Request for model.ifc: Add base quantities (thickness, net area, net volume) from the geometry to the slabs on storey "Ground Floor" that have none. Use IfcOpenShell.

First a look at what the model holds.

```python
import ifcopenshell
import ifcopenshell.util.element
import ifcopenshell.util.unit

model = ifcopenshell.open("model.ifc")
print(model.schema)
for unit_type in ("LENGTHUNIT", "AREAUNIT", "VOLUMEUNIT"):
    print(unit_type, ifcopenshell.util.unit.calculate_unit_scale(model, unit_type))
storey = next(s for s in model.by_type("IfcBuildingStorey") if s.Name == "Ground Floor")
slabs = [e for e in ifcopenshell.util.element.get_decomposition(storey) if e.is_a("IfcSlab")]
for e in sorted(slabs, key=lambda e: e.id()):
    print(e.id(), e.is_a(), e.Name, list(ifcopenshell.util.element.get_psets(e, qtos_only=True)), sep=" | ")
```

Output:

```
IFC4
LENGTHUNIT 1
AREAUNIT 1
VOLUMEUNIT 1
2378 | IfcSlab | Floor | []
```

```python
import ifcopenshell
import ifcopenshell.api.pset
import ifcopenshell.geom
import ifcopenshell.util.element
import ifcopenshell.util.shape
import ifcopenshell.util.unit

model = ifcopenshell.open("model.ifc")
unit_scale = ifcopenshell.util.unit.calculate_unit_scale(model)
area_scale = ifcopenshell.util.unit.calculate_unit_scale(model, "AREAUNIT")
volume_scale = ifcopenshell.util.unit.calculate_unit_scale(model, "VOLUMEUNIT")
settings = ifcopenshell.geom.settings()

storey = next(s for s in model.by_type("IfcBuildingStorey") if s.Name == "Ground Floor")
slabs = [e for e in ifcopenshell.util.element.get_decomposition(storey) if e.is_a("IfcSlab")]

for e in sorted(slabs, key=lambda e: e.id()):
    if ifcopenshell.util.element.get_psets(e, qtos_only=True, should_inherit=False):
        continue
    # Geometry comes back in metres, in the element's own axes.
    shape = ifcopenshell.geom.create_shape(settings, e)
    values = {
        "Width": ifcopenshell.util.shape.get_z(shape.geometry) / unit_scale,
        "NetArea": ifcopenshell.util.shape.get_footprint_area(shape.geometry) / area_scale,
        "NetVolume": ifcopenshell.util.shape.get_volume(shape.geometry) / volume_scale,
    }
    qto = ifcopenshell.api.pset.add_qto(model, product=e, name="Qto_SlabBaseQuantities")
    ifcopenshell.api.pset.edit_qto(model, qto=qto, properties=values)
    print(e.id(), {k: round(v, 3) for k, v in values.items()})

model.write("model_rev.ifc")
```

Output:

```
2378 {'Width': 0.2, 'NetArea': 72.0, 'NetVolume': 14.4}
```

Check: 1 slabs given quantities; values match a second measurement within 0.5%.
